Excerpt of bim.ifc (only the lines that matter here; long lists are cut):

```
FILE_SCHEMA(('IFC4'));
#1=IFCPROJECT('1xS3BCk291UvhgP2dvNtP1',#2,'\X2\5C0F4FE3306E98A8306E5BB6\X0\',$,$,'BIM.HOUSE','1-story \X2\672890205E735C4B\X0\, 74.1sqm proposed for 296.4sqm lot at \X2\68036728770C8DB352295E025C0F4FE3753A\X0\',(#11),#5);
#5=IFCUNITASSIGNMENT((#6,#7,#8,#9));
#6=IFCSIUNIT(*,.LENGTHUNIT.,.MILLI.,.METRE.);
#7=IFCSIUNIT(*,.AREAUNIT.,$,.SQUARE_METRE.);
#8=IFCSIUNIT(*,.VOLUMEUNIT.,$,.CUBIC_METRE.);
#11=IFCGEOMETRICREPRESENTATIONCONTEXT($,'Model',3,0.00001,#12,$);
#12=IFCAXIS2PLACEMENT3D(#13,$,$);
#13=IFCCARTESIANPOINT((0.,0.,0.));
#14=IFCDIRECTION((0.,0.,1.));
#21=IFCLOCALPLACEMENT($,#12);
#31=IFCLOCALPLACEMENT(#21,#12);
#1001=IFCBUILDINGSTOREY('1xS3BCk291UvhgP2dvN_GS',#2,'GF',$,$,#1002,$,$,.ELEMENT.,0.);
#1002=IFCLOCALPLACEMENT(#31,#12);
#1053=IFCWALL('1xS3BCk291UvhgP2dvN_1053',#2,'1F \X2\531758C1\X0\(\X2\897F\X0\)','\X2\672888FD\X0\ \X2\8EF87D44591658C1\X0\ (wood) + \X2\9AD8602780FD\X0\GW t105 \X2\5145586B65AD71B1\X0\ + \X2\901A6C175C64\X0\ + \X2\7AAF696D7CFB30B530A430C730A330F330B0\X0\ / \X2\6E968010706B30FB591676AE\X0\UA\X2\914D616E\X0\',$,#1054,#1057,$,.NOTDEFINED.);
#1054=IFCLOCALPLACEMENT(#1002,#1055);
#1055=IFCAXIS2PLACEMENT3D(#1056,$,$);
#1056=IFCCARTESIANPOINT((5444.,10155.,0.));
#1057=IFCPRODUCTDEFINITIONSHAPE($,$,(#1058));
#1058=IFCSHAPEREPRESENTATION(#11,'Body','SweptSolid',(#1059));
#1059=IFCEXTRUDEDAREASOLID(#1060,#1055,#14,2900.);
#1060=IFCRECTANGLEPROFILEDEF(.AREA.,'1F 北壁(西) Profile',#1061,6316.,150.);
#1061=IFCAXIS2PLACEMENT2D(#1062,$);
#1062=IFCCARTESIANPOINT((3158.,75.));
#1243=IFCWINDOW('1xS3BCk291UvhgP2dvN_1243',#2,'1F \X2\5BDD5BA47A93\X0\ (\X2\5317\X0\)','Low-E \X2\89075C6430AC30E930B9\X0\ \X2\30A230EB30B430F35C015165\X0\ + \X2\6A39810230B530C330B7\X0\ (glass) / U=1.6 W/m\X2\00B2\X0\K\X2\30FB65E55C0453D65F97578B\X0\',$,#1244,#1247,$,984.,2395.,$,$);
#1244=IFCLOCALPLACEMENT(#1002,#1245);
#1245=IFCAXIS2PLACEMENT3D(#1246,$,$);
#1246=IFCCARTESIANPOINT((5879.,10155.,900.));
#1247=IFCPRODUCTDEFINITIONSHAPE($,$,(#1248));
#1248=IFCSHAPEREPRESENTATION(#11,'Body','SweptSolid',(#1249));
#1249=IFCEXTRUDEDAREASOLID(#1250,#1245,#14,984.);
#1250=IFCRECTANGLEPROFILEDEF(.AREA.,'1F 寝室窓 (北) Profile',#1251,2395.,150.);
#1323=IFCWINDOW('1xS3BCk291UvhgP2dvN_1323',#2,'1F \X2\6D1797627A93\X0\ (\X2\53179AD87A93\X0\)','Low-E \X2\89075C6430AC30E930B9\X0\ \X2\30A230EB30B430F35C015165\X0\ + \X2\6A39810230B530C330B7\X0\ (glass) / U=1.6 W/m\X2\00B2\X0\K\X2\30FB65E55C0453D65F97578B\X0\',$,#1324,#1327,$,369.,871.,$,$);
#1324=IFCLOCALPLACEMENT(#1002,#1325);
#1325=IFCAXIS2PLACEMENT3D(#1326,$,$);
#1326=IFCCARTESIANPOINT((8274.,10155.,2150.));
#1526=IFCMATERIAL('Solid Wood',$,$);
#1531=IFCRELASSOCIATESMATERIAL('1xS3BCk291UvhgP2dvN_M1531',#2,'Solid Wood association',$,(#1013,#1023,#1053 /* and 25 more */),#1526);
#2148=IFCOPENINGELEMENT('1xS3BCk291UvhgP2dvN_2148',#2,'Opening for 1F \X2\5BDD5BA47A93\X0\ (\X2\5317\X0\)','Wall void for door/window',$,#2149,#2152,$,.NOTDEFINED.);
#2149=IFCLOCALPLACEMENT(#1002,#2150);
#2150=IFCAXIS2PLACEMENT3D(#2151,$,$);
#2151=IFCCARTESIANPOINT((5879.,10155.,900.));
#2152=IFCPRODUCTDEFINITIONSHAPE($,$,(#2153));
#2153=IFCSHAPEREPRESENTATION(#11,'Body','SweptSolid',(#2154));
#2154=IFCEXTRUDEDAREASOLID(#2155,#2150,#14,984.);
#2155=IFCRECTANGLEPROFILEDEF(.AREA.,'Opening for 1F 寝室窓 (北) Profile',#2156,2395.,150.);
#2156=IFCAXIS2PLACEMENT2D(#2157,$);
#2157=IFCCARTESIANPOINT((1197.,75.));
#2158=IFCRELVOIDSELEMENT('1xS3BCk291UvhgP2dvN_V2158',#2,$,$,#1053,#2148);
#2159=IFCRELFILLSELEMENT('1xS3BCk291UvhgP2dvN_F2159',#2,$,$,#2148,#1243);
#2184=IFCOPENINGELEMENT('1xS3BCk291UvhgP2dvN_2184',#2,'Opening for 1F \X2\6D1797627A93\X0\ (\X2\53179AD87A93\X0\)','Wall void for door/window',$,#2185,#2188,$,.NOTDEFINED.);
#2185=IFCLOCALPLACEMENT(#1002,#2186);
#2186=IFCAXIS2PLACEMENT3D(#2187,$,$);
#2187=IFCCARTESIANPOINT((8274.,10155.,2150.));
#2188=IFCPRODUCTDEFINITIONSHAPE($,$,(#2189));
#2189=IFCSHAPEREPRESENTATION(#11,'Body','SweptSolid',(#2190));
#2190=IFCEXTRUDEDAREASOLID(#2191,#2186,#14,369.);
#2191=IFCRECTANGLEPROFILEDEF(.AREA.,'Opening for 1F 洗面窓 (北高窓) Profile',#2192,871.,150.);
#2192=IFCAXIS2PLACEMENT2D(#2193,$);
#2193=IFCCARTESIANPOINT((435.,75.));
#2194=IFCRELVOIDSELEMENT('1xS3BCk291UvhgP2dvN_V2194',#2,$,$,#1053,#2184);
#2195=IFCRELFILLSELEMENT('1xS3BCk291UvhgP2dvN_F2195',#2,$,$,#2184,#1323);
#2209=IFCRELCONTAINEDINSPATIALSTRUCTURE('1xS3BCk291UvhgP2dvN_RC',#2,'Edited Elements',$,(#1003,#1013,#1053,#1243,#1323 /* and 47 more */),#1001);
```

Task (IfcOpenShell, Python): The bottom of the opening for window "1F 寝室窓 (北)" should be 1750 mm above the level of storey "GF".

```python
import numpy as np
import ifcopenshell
import ifcopenshell.api.geometry
import ifcopenshell.geom
import ifcopenshell.util.element
import ifcopenshell.util.placement
import ifcopenshell.util.shape
import ifcopenshell.util.unit

model = ifcopenshell.open("bim.ifc")
unit_scale = ifcopenshell.util.unit.calculate_unit_scale(model)

window = model.by_guid("1xS3BCk291UvhgP2dvN_1243")
opening = window.FillsVoids[0].RelatingOpeningElement
storey = ifcopenshell.util.element.get_container(window, ifc_class="IfcBuildingStorey")
level = ifcopenshell.util.placement.get_local_placement(storey.ObjectPlacement)[2, 3]

# The opening's origin need not be at the sill, so measure its lowest point.
shape = ifcopenshell.geom.create_shape(ifcopenshell.geom.settings(), opening)
bottom = ifcopenshell.util.shape.get_shape_bottom_elevation(shape, shape.geometry) / unit_scale
dz = level + 1750.0 - bottom

shift = np.array([0.0, 0.0, dz])
# The window is not placed relative to its opening, so move both.
for product in (opening, window):
    matrix = ifcopenshell.util.placement.get_local_placement(product.ObjectPlacement)
    matrix[:3, 3] += shift
    ifcopenshell.api.geometry.edit_object_placement(model, product=product, matrix=matrix, is_si=False)

print(f"moved by {dz * unit_scale:+.3f} m")

model.write("bim_rev.ifc")
```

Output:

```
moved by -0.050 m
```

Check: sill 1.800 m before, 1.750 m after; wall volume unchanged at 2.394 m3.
